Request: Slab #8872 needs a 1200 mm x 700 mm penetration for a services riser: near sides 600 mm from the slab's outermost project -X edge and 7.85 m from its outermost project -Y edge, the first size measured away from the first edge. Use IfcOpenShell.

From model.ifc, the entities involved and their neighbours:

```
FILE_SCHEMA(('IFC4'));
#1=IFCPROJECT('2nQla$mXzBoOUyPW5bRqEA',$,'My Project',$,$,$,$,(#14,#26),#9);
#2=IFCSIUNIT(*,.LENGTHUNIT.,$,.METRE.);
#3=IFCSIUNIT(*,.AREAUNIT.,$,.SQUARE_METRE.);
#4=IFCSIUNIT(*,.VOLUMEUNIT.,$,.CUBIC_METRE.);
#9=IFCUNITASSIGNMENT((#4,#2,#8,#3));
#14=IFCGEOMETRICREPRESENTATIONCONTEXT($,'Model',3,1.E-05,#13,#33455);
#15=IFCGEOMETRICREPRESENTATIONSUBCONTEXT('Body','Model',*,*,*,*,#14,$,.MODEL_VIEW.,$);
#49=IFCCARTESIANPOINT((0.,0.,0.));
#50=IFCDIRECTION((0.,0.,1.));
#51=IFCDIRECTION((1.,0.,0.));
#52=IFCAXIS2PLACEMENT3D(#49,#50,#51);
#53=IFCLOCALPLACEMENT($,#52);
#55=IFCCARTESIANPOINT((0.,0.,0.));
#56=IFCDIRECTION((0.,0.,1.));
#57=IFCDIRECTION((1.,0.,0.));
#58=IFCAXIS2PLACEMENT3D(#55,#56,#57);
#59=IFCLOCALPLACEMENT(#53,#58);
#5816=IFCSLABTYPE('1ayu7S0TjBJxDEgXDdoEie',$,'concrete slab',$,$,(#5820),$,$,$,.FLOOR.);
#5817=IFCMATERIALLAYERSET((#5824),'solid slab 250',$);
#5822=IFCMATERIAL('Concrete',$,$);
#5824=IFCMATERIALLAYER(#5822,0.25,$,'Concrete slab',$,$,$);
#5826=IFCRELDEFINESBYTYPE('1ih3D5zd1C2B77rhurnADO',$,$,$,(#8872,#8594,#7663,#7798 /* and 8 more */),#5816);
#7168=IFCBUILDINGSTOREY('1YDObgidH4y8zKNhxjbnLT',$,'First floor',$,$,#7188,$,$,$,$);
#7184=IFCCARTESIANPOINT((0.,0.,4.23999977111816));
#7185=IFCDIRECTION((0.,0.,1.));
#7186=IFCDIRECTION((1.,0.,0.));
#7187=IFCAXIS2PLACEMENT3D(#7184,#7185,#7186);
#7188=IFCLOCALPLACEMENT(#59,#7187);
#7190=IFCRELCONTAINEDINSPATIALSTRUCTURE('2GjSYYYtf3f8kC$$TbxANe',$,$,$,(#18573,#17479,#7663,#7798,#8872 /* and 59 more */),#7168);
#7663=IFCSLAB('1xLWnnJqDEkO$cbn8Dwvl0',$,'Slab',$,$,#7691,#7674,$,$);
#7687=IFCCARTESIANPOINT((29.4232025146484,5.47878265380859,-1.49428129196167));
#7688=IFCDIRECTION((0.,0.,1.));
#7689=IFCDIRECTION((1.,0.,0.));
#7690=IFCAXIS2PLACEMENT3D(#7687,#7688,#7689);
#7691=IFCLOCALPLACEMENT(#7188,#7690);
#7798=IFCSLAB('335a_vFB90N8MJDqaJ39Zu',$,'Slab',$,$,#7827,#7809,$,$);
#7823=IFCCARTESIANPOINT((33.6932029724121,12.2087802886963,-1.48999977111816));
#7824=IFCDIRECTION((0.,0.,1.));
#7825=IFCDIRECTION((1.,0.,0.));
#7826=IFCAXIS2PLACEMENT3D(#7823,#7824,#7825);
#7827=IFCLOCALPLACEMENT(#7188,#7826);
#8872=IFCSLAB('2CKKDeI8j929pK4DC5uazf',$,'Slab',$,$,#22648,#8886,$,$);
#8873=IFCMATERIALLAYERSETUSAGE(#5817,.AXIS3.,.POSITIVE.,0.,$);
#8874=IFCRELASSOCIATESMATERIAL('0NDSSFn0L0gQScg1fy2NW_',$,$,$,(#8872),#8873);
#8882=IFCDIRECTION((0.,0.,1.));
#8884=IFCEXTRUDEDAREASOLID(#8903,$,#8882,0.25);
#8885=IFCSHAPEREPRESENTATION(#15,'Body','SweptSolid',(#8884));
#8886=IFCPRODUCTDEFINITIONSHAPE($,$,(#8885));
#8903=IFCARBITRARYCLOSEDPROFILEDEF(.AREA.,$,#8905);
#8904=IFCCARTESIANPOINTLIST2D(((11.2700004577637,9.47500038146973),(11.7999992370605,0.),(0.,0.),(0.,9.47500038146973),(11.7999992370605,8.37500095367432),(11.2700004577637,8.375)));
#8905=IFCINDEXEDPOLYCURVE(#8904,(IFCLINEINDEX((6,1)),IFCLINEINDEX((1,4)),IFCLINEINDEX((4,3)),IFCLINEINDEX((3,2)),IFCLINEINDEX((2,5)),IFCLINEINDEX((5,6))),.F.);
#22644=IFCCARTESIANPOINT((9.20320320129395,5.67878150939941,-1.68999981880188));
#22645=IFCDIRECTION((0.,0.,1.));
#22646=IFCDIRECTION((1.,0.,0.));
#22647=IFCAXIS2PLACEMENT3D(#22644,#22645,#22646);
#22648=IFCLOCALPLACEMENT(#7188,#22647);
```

```python
import numpy as np
import ifcopenshell
import ifcopenshell.api.feature
import ifcopenshell.api.geometry
import ifcopenshell.api.root
import ifcopenshell.geom
import ifcopenshell.util.placement
import ifcopenshell.util.representation
import ifcopenshell.util.shape
import ifcopenshell.util.unit

model = ifcopenshell.open("model.ifc")
unit_scale = ifcopenshell.util.unit.calculate_unit_scale(model)
settings = ifcopenshell.geom.settings()


def volume(element):
    """Net volume in cubic metres, openings subtracted."""
    shape = ifcopenshell.geom.create_shape(settings, element)
    return ifcopenshell.util.shape.get_volume(shape.geometry)


slab = model.by_guid("2CKKDeI8j929pK4DC5uazf")
before = volume(slab)

# Extent in the slab's own axes, in metres. The edges named are its -X and -Y sides.
slab_shape = ifcopenshell.geom.create_shape(settings, slab)
vertices = ifcopenshell.util.shape.get_vertices(slab_shape.geometry)
x_min, y_min, bottom = vertices.min(axis=0)
top = vertices[:, 2].max()

opening = ifcopenshell.api.root.create_entity(model, ifc_class="IfcOpeningElement", name="Services riser opening", predefined_type="OPENING")
context = ifcopenshell.util.representation.get_context(model, "Model", "Body", "MODEL_VIEW")
width, depth = 1.2, 0.7
outline = [(0.0, 0.0), (width, 0.0), (width, depth), (0.0, depth), (0.0, 0.0)]
# Overshoot both faces by 50 mm so the cut is clean.
shape = ifcopenshell.api.geometry.add_slab_representation(
    model, context=context, depth=top - bottom + 0.1, polyline=outline
)
ifcopenshell.api.geometry.assign_representation(model, product=opening, representation=shape)

matrix = ifcopenshell.util.placement.get_local_placement(slab.ObjectPlacement)
matrix[:, 3] = matrix @ np.append(np.array([x_min + 0.6, y_min + 7.85, bottom - 0.05]) / unit_scale, 1.0)
ifcopenshell.api.geometry.edit_object_placement(model, product=opening, matrix=matrix, is_si=False)
ifcopenshell.api.feature.add_feature(model, feature=opening, element=slab)

after = volume(slab)

print(f"slab volume {before:.3f} -> {after:.3f} m3")

model.write("model-out.ifc")
```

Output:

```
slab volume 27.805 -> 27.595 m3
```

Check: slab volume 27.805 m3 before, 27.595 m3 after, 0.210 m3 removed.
